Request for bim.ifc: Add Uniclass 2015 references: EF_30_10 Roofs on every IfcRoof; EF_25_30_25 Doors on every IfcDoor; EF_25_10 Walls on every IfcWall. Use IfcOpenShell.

First a look at what the model holds.

```python
import ifcopenshell

model = ifcopenshell.open("bim.ifc")
print(model.schema)
print("classifications:", [c.Name for c in model.by_type("IfcClassification")])
for ifc_class in ("IfcDoor", "IfcRoof", "IfcStair", "IfcWall", "IfcWindow"):
    print(ifc_class, len(model.by_type(ifc_class)))
```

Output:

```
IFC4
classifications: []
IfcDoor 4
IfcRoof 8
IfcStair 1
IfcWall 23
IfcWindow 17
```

```python
import ifcopenshell
import ifcopenshell.api.classification

model = ifcopenshell.open("bim.ifc")

system = ifcopenshell.api.classification.add_classification(model, classification="Uniclass 2015")

codes = {
    "IfcRoof": ("EF_30_10", "Roofs"),
    "IfcDoor": ("EF_25_30_25", "Doors"),
    "IfcWall": ("EF_25_10", "Walls"),
}
for ifc_class, (code, name) in codes.items():
    products = model.by_type(ifc_class)
    ifcopenshell.api.classification.add_reference(
        model, products=products, classification=system, identification=code, name=name
    )
    print(code, len(products))

model.write("bim_rev.ifc")
```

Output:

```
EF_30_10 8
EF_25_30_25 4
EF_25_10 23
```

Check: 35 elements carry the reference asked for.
